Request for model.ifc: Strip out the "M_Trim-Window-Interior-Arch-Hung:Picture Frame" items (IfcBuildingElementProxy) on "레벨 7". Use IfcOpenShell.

First a look at what the model holds.

```python
import ifcopenshell
import ifcopenshell.util.element

model = ifcopenshell.open("model.ifc")
print(model.schema)
storey = next(s for s in model.by_type("IfcBuildingStorey") if s.Name == "레벨 7")
proxies = [e for e in ifcopenshell.util.element.get_decomposition(storey) if e.is_a("IfcBuildingElementProxy")]
seen = {}
for e in proxies:
    element_type = ifcopenshell.util.element.get_type(e)
    name = element_type.Name if element_type not in (None, e) else None
    seen[name] = seen.get(name, 0) + 1
for name, count in sorted(seen.items(), key=str):
    print(count, "x", name)
```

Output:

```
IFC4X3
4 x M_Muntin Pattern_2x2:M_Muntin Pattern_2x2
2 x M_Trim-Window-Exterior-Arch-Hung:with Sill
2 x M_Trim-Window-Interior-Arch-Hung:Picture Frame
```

```python
import ifcopenshell
import ifcopenshell.api.root
import ifcopenshell.util.element

model = ifcopenshell.open("model.ifc")

storey = next(s for s in model.by_type("IfcBuildingStorey") if s.Name == "레벨 7")
proxies = [e for e in ifcopenshell.util.element.get_decomposition(storey) if e.is_a("IfcBuildingElementProxy")]
targets = [e for e in proxies if (t := ifcopenshell.util.element.get_type(e)) not in (None, e) and t.Name == "M_Trim-Window-Interior-Arch-Hung:Picture Frame"]

for e in targets:
    ifcopenshell.api.root.remove_product(model, product=e)
print(len(targets), "removed")

model.write("model-out.ifc")
```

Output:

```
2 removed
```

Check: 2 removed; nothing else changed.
